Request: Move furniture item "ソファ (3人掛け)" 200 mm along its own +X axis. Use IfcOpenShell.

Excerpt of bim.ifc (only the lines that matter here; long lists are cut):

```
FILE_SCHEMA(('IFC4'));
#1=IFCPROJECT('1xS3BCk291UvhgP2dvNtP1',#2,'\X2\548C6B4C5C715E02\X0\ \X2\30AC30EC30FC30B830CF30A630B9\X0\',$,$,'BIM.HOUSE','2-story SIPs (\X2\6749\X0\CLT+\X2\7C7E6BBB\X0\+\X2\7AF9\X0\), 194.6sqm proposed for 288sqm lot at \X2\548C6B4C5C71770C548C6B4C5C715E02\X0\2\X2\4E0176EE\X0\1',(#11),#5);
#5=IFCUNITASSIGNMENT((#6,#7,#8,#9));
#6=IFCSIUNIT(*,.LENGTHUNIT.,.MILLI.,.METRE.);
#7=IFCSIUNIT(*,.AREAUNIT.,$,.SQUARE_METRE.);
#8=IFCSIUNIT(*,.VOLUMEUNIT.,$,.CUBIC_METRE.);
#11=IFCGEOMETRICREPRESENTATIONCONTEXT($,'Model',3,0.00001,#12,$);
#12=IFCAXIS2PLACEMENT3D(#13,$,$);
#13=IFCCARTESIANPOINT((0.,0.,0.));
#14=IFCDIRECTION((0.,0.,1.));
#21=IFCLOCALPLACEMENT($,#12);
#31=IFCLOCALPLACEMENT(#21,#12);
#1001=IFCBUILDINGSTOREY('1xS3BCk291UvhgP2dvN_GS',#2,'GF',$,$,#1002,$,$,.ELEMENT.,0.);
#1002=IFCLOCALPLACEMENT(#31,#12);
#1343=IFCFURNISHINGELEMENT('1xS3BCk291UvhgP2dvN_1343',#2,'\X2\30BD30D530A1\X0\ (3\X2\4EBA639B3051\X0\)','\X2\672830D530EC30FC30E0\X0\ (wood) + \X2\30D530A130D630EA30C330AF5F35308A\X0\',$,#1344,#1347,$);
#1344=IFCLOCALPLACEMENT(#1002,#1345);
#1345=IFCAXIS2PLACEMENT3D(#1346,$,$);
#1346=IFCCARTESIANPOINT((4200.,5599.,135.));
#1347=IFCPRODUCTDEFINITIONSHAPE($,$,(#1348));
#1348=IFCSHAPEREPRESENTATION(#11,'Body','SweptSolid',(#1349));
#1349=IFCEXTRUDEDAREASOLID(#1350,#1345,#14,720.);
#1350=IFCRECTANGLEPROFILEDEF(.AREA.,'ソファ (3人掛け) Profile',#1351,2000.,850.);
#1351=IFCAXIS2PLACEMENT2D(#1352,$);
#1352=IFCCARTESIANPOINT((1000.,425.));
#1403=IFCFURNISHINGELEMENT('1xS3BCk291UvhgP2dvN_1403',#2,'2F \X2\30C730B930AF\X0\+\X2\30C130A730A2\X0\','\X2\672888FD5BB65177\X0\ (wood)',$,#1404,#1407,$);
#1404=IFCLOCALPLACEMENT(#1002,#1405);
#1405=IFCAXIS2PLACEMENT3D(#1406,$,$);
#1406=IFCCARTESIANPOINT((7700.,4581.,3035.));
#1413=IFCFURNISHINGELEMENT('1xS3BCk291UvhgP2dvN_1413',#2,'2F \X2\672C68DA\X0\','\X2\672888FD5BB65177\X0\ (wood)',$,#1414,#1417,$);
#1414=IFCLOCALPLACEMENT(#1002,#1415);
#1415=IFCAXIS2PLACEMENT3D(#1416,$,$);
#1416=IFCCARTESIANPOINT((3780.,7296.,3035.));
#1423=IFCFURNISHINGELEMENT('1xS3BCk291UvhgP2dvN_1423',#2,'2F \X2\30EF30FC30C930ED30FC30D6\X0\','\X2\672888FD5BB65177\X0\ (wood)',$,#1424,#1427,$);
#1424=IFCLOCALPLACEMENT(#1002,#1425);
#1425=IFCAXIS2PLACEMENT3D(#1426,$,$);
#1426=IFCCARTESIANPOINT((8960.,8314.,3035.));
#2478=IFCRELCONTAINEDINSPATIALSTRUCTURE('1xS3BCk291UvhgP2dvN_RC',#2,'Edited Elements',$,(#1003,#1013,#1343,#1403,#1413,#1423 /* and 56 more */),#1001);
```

```python
import ifcopenshell
import ifcopenshell.api.geometry
import ifcopenshell.util.placement
import ifcopenshell.util.unit

model = ifcopenshell.open("bim.ifc")
unit_scale = ifcopenshell.util.unit.calculate_unit_scale(model)

item = model.by_guid("1xS3BCk291UvhgP2dvN_1343")
matrix = ifcopenshell.util.placement.get_local_placement(item.ObjectPlacement)
matrix[:3, 3] += matrix[:3, 0] * 0.2 / unit_scale
ifcopenshell.api.geometry.edit_object_placement(model, product=item, matrix=matrix, is_si=False)

print(ifcopenshell.util.placement.get_local_placement(item.ObjectPlacement).round(3) + 0.0)

model.write("bim_rev.ifc")
```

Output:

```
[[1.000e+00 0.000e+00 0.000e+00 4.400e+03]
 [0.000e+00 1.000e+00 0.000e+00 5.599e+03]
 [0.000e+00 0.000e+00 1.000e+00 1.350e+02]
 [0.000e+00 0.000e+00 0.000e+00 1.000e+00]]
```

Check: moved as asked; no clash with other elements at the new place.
